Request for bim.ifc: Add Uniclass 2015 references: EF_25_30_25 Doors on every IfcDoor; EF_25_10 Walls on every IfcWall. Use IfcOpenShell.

First a look at what the model holds.

```python
import ifcopenshell

model = ifcopenshell.open("bim.ifc")
print(model.schema)
print("classifications:", [c.Name for c in model.by_type("IfcClassification")])
for ifc_class in ("IfcDoor", "IfcRoof", "IfcStair", "IfcWall", "IfcWindow"):
    print(ifc_class, len(model.by_type(ifc_class)))
```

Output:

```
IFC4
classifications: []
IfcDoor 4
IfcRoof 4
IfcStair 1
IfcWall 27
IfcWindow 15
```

```python
import ifcopenshell
import ifcopenshell.api.classification

model = ifcopenshell.open("bim.ifc")

system = ifcopenshell.api.classification.add_classification(model, classification="Uniclass 2015")

codes = {
    "IfcDoor": ("EF_25_30_25", "Doors"),
    "IfcWall": ("EF_25_10", "Walls"),
}
for ifc_class, (code, name) in codes.items():
    products = model.by_type(ifc_class)
    ifcopenshell.api.classification.add_reference(
        model, products=products, classification=system, identification=code, name=name
    )
    print(code, len(products))

model.write("bim_rev.ifc")
```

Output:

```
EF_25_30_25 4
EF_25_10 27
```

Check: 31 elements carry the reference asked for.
